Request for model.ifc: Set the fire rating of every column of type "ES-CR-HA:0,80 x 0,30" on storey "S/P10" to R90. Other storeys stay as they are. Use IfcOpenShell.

First a look at what the model holds.

```python
import ifcopenshell
import ifcopenshell.util.element

model = ifcopenshell.open("model.ifc")
print(model.schema)
storey = next(s for s in model.by_type("IfcBuildingStorey") if s.Name == "S/P10")
columns = [e for e in ifcopenshell.util.element.get_decomposition(storey) if e.is_a("IfcColumn")]
seen = {}
for e in columns:
    element_type = ifcopenshell.util.element.get_type(e)
    key = (element_type.Name if element_type != e and element_type else None, ifcopenshell.util.element.get_pset(e, "Pset_ColumnCommon", "FireRating"))
    seen[key] = seen.get(key, 0) + 1
for (name, value), count in sorted(seen.items(), key=str):
    print(count, "x", name, "|", value)
```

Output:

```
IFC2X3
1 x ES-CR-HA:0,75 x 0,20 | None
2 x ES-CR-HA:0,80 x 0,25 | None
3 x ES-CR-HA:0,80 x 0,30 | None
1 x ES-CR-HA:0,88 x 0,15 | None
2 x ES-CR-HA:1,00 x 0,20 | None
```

```python
import ifcopenshell
import ifcopenshell.api.pset
import ifcopenshell.util.element

model = ifcopenshell.open("model.ifc")

storey = next(s for s in model.by_type("IfcBuildingStorey") if s.Name == "S/P10")
columns = [e for e in ifcopenshell.util.element.get_decomposition(storey) if e.is_a("IfcColumn")]

count = 0
for e in columns:
    element_type = ifcopenshell.util.element.get_type(e)
    if element_type in (None, e) or element_type.Name != "ES-CR-HA:0,80 x 0,30":
        continue
    # add_pset returns the element's existing set when there is one.
    pset = ifcopenshell.api.pset.add_pset(model, product=e, name="Pset_ColumnCommon")
    ifcopenshell.api.pset.edit_pset(model, pset=pset, properties={"FireRating": "R90"})
    count += 1

print(count, "columns updated")

model.write("model-out.ifc")
```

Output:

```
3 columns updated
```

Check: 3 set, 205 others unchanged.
